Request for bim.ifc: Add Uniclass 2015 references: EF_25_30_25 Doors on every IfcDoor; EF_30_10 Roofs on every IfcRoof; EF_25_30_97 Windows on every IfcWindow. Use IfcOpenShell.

First a look at what the model holds.

```python
import ifcopenshell

model = ifcopenshell.open("bim.ifc")
print(model.schema)
print("classifications:", [c.Name for c in model.by_type("IfcClassification")])
for ifc_class in ("IfcDoor", "IfcRoof", "IfcStair", "IfcWall", "IfcWindow"):
    print(ifc_class, len(model.by_type(ifc_class)))
```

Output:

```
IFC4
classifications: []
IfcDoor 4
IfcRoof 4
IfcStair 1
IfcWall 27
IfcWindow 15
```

```python
import ifcopenshell
import ifcopenshell.api.classification

model = ifcopenshell.open("bim.ifc")

system = ifcopenshell.api.classification.add_classification(model, classification="Uniclass 2015")

codes = {
    "IfcDoor": ("EF_25_30_25", "Doors"),
    "IfcRoof": ("EF_30_10", "Roofs"),
    "IfcWindow": ("EF_25_30_97", "Windows"),
}
for ifc_class, (code, name) in codes.items():
    products = model.by_type(ifc_class)
    ifcopenshell.api.classification.add_reference(
        model, products=products, classification=system, identification=code, name=name
    )
    print(code, len(products))

model.write("bim-out.ifc")
```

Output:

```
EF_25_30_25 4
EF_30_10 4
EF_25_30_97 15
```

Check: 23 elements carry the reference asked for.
